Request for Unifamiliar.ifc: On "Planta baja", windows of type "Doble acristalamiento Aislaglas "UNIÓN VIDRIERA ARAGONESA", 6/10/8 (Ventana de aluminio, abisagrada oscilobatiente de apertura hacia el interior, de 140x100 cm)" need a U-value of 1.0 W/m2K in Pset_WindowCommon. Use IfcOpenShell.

First a look at what the model holds.

```python
import ifcopenshell
import ifcopenshell.util.element

model = ifcopenshell.open("Unifamiliar.ifc")
print(model.schema)
storey = next(s for s in model.by_type("IfcBuildingStorey") if s.Name == "Planta baja")
windows = [e for e in ifcopenshell.util.element.get_decomposition(storey) if e.is_a("IfcWindow")]
seen = {}
for e in windows:
    element_type = ifcopenshell.util.element.get_type(e)
    key = (element_type.Name if element_type != e and element_type else None, ifcopenshell.util.element.get_pset(e, "Pset_WindowCommon", "ThermalTransmittance"))
    seen[key] = seen.get(key, 0) + 1
for (name, value), count in sorted(seen.items(), key=str):
    print(count, "x", name, "|", value)
```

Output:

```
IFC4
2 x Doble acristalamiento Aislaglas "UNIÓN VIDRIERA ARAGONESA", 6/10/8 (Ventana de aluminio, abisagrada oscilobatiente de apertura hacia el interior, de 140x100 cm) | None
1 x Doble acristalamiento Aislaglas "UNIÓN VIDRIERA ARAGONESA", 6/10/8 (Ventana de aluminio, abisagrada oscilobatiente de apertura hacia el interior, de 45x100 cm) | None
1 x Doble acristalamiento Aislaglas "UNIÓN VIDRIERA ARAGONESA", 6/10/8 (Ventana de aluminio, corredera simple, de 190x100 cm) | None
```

```python
import ifcopenshell
import ifcopenshell.api.pset
import ifcopenshell.util.element

model = ifcopenshell.open("Unifamiliar.ifc")

storey = next(s for s in model.by_type("IfcBuildingStorey") if s.Name == "Planta baja")
windows = [e for e in ifcopenshell.util.element.get_decomposition(storey) if e.is_a("IfcWindow")]

count = 0
for e in windows:
    element_type = ifcopenshell.util.element.get_type(e)
    if element_type in (None, e) or element_type.Name != 'Doble acristalamiento Aislaglas "UNIÓN VIDRIERA ARAGONESA", 6/10/8 (Ventana de aluminio, abisagrada oscilobatiente de apertura hacia el interior, de 140x100 cm)':
        continue
    # add_pset returns the element's existing set when there is one.
    pset = ifcopenshell.api.pset.add_pset(model, product=e, name="Pset_WindowCommon")
    ifcopenshell.api.pset.edit_pset(model, pset=pset, properties={"ThermalTransmittance": 1.0})
    count += 1

print(count, "windows updated")

model.write("Unifamiliar_updated.ifc")
```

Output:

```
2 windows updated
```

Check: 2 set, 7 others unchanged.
